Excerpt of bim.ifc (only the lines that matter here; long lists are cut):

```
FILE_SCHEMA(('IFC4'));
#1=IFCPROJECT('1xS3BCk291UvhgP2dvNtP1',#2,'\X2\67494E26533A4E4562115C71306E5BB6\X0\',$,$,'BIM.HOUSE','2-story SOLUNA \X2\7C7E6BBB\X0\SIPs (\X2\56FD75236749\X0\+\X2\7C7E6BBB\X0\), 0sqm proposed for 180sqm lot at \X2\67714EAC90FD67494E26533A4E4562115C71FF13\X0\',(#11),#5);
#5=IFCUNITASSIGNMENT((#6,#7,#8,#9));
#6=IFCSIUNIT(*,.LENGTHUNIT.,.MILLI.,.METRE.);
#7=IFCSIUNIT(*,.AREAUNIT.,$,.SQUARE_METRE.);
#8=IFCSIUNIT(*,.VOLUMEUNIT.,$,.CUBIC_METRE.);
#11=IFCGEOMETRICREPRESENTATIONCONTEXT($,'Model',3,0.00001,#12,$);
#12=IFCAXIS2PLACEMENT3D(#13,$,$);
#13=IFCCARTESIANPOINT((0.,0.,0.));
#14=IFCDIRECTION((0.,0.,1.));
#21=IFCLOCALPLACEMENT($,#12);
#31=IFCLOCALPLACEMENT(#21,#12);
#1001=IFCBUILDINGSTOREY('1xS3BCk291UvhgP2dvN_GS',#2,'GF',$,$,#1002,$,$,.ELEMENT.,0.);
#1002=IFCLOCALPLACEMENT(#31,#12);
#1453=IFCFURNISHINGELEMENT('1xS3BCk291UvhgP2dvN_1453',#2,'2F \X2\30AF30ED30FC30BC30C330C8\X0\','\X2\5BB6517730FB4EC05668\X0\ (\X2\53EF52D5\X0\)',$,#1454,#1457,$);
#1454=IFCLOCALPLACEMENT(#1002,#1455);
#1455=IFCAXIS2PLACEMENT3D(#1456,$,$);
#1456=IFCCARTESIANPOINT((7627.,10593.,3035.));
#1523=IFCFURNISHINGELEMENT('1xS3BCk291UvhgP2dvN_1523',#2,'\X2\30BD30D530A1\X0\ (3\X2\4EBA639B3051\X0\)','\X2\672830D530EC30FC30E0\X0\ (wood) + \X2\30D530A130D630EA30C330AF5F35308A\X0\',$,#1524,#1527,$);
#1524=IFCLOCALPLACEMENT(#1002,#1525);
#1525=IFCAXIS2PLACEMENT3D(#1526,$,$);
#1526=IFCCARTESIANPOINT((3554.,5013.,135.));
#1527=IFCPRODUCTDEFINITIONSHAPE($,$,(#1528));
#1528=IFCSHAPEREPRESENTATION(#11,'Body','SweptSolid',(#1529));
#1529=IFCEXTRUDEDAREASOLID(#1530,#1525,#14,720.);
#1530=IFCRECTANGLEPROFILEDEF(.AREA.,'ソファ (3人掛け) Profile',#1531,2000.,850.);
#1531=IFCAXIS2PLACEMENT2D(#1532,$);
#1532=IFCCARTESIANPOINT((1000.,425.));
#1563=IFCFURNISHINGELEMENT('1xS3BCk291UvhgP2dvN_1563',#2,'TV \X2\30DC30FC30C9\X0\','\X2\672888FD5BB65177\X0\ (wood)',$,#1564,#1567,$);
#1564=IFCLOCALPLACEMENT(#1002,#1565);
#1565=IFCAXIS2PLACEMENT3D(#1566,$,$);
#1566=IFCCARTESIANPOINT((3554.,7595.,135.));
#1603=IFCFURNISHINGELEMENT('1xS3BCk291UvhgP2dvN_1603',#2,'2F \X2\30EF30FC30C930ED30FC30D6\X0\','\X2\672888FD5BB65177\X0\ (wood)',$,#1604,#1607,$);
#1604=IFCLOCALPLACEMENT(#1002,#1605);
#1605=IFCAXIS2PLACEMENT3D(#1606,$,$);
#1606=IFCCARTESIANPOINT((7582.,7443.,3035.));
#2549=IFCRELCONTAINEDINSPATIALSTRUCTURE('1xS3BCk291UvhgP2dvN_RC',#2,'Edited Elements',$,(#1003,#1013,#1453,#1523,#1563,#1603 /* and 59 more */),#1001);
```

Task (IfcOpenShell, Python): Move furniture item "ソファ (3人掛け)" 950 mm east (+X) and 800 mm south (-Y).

```python
import ifcopenshell
import ifcopenshell.api.geometry
import ifcopenshell.util.placement
import ifcopenshell.util.unit

model = ifcopenshell.open("bim.ifc")
unit_scale = ifcopenshell.util.unit.calculate_unit_scale(model)

item = model.by_guid("1xS3BCk291UvhgP2dvN_1523")
matrix = ifcopenshell.util.placement.get_local_placement(item.ObjectPlacement)
matrix[0, 3] += 0.95 / unit_scale
matrix[1, 3] -= 0.8 / unit_scale
ifcopenshell.api.geometry.edit_object_placement(model, product=item, matrix=matrix, is_si=False)

print(ifcopenshell.util.placement.get_local_placement(item.ObjectPlacement).round(3) + 0.0)

model.write("bim_rev.ifc")
```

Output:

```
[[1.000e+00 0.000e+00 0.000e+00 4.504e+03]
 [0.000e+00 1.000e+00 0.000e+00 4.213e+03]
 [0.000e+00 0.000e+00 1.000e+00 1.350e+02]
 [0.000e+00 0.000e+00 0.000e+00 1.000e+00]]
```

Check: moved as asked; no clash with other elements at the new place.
